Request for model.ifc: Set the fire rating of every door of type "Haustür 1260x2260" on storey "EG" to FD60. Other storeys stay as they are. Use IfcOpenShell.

First a look at what the model holds.

```python
import ifcopenshell
import ifcopenshell.util.element

model = ifcopenshell.open("model.ifc")
print(model.schema)
storey = next(s for s in model.by_type("IfcBuildingStorey") if s.Name == "EG")
doors = [e for e in ifcopenshell.util.element.get_decomposition(storey) if e.is_a("IfcDoor")]
seen = {}
for e in doors:
    element_type = ifcopenshell.util.element.get_type(e)
    key = (element_type.Name if element_type != e and element_type else None, ifcopenshell.util.element.get_pset(e, "Pset_DoorCommon", "FireRating"))
    seen[key] = seen.get(key, 0) + 1
for (name, value), count in sorted(seen.items(), key=str):
    print(count, "x", name, "|", value)
```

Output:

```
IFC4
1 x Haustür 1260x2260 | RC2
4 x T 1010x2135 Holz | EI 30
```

```python
import ifcopenshell
import ifcopenshell.api.pset
import ifcopenshell.util.element

model = ifcopenshell.open("model.ifc")

storey = next(s for s in model.by_type("IfcBuildingStorey") if s.Name == "EG")
doors = [e for e in ifcopenshell.util.element.get_decomposition(storey) if e.is_a("IfcDoor")]

count = 0
for e in doors:
    element_type = ifcopenshell.util.element.get_type(e)
    if element_type in (None, e) or element_type.Name != "Haustür 1260x2260":
        continue
    # add_pset returns the element's existing set when there is one.
    pset = ifcopenshell.api.pset.add_pset(model, product=e, name="Pset_DoorCommon")
    ifcopenshell.api.pset.edit_pset(model, pset=pset, properties={"FireRating": "FD60"})
    count += 1

print(count, "doors updated")

model.write("model_v2.ifc")
```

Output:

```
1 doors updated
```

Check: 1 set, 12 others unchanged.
